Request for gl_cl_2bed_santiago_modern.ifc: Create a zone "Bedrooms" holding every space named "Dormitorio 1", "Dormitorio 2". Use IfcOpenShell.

First a look at what the model holds.

```python
import ifcopenshell

model = ifcopenshell.open("gl_cl_2bed_santiago_modern.ifc")
print(model.schema)
seen = {}
for space in model.by_type("IfcSpace"):
    seen[space.LongName] = seen.get(space.LongName, 0) + 1
for name, count in sorted(seen.items(), key=str):
    print(count, "x", name)
print("zones:", [z.Name for z in model.by_type("IfcZone")][:20])
```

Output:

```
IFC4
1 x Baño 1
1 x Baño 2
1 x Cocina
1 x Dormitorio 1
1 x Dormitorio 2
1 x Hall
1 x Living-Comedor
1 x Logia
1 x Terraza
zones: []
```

```python
import ifcopenshell
import ifcopenshell.api.group
import ifcopenshell.api.root

model = ifcopenshell.open("gl_cl_2bed_santiago_modern.ifc")

names = {"Dormitorio 1", "Dormitorio 2"}
spaces = [s for s in model.by_type("IfcSpace") if s.LongName in names]

zone = ifcopenshell.api.root.create_entity(model, ifc_class="IfcZone", name="Bedrooms")
ifcopenshell.api.group.assign_group(model, products=spaces, group=zone)
print(len(spaces), "spaces in", zone.Name)

model.write("gl_cl_2bed_santiago_modern_updated.ifc")
```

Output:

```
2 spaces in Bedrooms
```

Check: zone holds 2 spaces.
